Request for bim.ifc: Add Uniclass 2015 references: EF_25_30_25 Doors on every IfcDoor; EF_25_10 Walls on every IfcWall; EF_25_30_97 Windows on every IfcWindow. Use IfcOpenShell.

First a look at what the model holds.

```python
import ifcopenshell

model = ifcopenshell.open("bim.ifc")
print(model.schema)
print("classifications:", [c.Name for c in model.by_type("IfcClassification")])
for ifc_class in ("IfcDoor", "IfcRoof", "IfcStair", "IfcWall", "IfcWindow"):
    print(ifc_class, len(model.by_type(ifc_class)))
```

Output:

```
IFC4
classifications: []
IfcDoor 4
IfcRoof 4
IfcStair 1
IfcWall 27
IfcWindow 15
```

```python
import ifcopenshell
import ifcopenshell.api.classification

model = ifcopenshell.open("bim.ifc")

system = ifcopenshell.api.classification.add_classification(model, classification="Uniclass 2015")

codes = {
    "IfcDoor": ("EF_25_30_25", "Doors"),
    "IfcWall": ("EF_25_10", "Walls"),
    "IfcWindow": ("EF_25_30_97", "Windows"),
}
for ifc_class, (code, name) in codes.items():
    products = model.by_type(ifc_class)
    ifcopenshell.api.classification.add_reference(
        model, products=products, classification=system, identification=code, name=name
    )
    print(code, len(products))

model.write("bim_edited.ifc")
```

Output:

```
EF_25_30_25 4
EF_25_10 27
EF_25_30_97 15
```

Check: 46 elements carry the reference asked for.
